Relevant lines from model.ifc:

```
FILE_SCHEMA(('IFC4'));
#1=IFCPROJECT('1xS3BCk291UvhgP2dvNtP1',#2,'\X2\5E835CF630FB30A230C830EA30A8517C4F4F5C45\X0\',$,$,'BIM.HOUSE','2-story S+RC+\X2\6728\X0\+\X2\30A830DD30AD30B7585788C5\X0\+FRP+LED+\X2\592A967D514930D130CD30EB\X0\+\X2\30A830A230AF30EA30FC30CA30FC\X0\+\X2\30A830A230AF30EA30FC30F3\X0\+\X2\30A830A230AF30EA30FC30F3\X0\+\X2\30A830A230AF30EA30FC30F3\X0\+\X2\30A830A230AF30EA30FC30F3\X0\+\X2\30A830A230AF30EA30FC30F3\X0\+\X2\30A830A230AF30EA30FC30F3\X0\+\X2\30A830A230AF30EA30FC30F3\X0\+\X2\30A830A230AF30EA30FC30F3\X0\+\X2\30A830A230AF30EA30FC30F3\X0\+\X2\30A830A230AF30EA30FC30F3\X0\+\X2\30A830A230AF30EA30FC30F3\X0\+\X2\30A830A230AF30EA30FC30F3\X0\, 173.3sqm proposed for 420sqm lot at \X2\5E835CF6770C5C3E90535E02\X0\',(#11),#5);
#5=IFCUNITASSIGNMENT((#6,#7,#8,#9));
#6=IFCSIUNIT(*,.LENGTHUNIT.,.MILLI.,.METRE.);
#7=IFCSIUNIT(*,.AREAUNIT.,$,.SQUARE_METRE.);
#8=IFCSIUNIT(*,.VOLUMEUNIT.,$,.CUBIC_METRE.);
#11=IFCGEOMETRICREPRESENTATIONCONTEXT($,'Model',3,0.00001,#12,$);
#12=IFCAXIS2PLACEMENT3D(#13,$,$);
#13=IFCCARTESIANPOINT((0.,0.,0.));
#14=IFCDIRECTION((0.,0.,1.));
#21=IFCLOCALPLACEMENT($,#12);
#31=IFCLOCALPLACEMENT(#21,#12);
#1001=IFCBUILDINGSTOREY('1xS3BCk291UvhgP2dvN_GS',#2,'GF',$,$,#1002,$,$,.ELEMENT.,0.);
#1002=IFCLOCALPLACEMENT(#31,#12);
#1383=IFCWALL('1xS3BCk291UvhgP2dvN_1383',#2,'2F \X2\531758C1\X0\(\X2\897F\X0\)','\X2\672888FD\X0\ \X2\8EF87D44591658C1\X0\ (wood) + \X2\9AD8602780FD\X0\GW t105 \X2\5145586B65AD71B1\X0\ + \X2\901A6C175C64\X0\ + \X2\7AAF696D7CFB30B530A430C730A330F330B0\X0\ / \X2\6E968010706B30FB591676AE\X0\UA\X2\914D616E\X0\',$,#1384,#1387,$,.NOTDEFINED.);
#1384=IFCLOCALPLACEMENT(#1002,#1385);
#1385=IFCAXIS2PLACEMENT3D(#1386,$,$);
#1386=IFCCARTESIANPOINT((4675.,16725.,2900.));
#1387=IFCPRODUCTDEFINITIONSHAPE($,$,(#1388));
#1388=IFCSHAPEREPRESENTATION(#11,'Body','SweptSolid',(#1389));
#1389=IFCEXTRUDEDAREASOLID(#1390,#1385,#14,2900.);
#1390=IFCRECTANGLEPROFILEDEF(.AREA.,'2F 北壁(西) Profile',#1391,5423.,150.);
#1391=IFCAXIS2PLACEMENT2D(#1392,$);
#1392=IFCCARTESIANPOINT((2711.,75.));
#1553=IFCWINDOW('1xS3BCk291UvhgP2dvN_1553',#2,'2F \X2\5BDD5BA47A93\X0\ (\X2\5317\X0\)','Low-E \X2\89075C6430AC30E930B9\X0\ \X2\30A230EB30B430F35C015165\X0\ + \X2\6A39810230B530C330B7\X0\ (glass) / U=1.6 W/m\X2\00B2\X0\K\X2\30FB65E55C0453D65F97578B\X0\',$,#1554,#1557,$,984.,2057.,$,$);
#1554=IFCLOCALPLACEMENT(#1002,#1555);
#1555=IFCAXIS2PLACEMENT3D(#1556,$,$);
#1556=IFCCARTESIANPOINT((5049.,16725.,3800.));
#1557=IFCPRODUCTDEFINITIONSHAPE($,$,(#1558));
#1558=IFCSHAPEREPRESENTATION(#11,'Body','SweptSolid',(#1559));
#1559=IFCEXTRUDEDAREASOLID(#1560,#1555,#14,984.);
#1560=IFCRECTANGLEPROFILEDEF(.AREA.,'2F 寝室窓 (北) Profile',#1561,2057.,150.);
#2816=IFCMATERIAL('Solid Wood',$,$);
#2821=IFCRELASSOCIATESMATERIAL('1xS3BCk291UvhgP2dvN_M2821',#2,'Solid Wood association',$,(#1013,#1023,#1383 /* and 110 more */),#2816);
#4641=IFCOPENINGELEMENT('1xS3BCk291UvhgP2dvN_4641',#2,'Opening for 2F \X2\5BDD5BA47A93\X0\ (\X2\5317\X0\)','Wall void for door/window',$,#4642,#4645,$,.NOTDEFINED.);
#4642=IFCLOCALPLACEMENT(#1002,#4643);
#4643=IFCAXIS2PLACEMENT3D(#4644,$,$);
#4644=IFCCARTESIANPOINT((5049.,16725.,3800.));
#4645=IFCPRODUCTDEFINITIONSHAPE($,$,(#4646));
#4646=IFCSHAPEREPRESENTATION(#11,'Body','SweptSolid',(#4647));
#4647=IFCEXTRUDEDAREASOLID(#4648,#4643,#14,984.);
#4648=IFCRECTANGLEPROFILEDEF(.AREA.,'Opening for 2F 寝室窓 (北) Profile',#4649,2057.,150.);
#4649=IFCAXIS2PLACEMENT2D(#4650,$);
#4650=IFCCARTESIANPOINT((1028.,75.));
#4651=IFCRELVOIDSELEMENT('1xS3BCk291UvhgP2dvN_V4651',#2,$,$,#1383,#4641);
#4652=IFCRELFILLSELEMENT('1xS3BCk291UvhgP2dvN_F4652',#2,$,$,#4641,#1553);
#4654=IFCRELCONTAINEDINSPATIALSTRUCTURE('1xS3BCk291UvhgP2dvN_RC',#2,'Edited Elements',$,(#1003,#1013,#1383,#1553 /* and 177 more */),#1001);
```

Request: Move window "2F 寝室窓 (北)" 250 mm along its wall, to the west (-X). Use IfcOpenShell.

```python
import ifcopenshell
import ifcopenshell.api.geometry
import ifcopenshell.util.placement
import ifcopenshell.util.unit

model = ifcopenshell.open("model.ifc")
unit_scale = ifcopenshell.util.unit.calculate_unit_scale(model)

window = model.by_guid("1xS3BCk291UvhgP2dvN_1553")
opening = window.FillsVoids[0].RelatingOpeningElement
wall = opening.VoidsElements[0].RelatingBuildingElement

wall_matrix = ifcopenshell.util.placement.get_local_placement(wall.ObjectPlacement)
shift = wall_matrix[:3, 0] * -0.25 / unit_scale
before = ifcopenshell.util.placement.get_local_placement(window.ObjectPlacement)[:3, 3].copy()

# The window is not placed relative to its opening, so move both.
for product in (opening, window):
    matrix = ifcopenshell.util.placement.get_local_placement(product.ObjectPlacement)
    matrix[:3, 3] += shift
    ifcopenshell.api.geometry.edit_object_placement(model, product=product, matrix=matrix, is_si=False)

after = ifcopenshell.util.placement.get_local_placement(window.ObjectPlacement)[:3, 3]
print("window moved by", (after - before).round(3) + 0.0)

model.write("model_edited.ifc")
```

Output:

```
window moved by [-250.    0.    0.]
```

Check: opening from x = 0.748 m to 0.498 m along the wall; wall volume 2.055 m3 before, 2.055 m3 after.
